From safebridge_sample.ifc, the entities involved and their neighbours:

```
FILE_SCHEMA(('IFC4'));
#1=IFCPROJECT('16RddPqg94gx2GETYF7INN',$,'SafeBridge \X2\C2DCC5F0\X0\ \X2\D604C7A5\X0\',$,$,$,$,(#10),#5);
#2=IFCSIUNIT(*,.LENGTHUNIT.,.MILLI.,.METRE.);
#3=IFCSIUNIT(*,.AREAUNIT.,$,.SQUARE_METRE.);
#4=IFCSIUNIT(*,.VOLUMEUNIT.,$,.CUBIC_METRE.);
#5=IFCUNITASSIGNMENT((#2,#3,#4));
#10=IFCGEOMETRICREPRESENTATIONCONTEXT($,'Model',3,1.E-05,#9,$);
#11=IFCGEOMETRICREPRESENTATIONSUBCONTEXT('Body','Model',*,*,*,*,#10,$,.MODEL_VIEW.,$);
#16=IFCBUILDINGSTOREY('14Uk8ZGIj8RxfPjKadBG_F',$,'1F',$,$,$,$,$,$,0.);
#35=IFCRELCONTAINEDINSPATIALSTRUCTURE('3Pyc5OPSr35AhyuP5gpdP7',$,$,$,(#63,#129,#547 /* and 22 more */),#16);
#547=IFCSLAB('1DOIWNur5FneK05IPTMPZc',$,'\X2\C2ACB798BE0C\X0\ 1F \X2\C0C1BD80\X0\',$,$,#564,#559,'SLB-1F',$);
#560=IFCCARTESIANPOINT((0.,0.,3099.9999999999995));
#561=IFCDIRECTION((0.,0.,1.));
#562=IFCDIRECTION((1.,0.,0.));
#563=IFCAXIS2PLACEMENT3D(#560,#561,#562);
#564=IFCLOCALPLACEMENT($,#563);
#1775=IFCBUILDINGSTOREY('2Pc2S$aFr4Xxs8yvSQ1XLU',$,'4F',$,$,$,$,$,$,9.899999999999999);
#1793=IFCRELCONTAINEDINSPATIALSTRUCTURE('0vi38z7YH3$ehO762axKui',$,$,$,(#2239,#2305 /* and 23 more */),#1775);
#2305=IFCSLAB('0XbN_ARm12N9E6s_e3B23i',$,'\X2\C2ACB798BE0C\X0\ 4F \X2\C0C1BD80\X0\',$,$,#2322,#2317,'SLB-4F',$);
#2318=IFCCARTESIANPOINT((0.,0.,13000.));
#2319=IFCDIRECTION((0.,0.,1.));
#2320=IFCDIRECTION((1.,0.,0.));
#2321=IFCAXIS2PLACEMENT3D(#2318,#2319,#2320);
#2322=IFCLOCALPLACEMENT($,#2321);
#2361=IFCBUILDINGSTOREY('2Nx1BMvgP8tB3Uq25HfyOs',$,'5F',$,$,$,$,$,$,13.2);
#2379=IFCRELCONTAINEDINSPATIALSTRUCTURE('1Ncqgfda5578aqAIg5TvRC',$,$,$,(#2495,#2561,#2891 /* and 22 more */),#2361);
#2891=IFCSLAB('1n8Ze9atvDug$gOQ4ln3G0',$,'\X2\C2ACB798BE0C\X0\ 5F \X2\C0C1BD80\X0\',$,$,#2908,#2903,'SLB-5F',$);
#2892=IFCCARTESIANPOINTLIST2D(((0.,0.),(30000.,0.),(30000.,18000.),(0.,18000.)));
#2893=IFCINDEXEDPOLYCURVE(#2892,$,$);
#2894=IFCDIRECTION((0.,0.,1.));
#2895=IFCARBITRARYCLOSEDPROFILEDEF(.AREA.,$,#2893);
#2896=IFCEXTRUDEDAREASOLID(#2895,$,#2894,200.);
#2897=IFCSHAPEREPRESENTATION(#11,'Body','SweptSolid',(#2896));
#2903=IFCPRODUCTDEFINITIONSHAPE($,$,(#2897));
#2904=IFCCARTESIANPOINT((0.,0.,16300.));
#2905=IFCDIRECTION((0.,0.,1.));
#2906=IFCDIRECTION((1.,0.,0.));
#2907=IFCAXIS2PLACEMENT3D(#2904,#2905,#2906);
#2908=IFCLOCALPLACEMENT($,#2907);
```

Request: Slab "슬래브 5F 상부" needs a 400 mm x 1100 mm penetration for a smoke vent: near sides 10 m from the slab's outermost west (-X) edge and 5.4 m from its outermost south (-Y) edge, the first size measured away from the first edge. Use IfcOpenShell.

```python
import numpy as np
import ifcopenshell
import ifcopenshell.api.feature
import ifcopenshell.api.geometry
import ifcopenshell.api.root
import ifcopenshell.geom
import ifcopenshell.util.placement
import ifcopenshell.util.representation
import ifcopenshell.util.shape
import ifcopenshell.util.unit

model = ifcopenshell.open("safebridge_sample.ifc")
unit_scale = ifcopenshell.util.unit.calculate_unit_scale(model)
settings = ifcopenshell.geom.settings()


def volume(element):
    """Net volume in cubic metres, openings subtracted."""
    shape = ifcopenshell.geom.create_shape(settings, element)
    return ifcopenshell.util.shape.get_volume(shape.geometry)


slab = model.by_id(2891)
before = volume(slab)

# Extent in the slab's own axes, in metres. The edges named are its -X and -Y sides.
slab_shape = ifcopenshell.geom.create_shape(settings, slab)
vertices = ifcopenshell.util.shape.get_vertices(slab_shape.geometry)
x_min, y_min, bottom = vertices.min(axis=0)
top = vertices[:, 2].max()

opening = ifcopenshell.api.root.create_entity(model, ifc_class="IfcOpeningElement", name="Smoke vent opening", predefined_type="OPENING")
context = ifcopenshell.util.representation.get_context(model, "Model", "Body", "MODEL_VIEW")
width, depth = 0.4, 1.1
outline = [(0.0, 0.0), (width, 0.0), (width, depth), (0.0, depth), (0.0, 0.0)]
# Overshoot both faces by 50 mm so the cut is clean.
shape = ifcopenshell.api.geometry.add_slab_representation(
    model, context=context, depth=top - bottom + 0.1, polyline=outline
)
ifcopenshell.api.geometry.assign_representation(model, product=opening, representation=shape)

matrix = ifcopenshell.util.placement.get_local_placement(slab.ObjectPlacement)
matrix[:, 3] = matrix @ np.append(np.array([x_min + 10, y_min + 5.4, bottom - 0.05]) / unit_scale, 1.0)
ifcopenshell.api.geometry.edit_object_placement(model, product=opening, matrix=matrix, is_si=False)
ifcopenshell.api.feature.add_feature(model, feature=opening, element=slab)

after = volume(slab)

print(f"slab volume {before:.3f} -> {after:.3f} m3")

model.write("safebridge_sample_rev.ifc")
```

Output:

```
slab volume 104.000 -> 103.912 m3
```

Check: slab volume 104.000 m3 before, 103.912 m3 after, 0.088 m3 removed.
